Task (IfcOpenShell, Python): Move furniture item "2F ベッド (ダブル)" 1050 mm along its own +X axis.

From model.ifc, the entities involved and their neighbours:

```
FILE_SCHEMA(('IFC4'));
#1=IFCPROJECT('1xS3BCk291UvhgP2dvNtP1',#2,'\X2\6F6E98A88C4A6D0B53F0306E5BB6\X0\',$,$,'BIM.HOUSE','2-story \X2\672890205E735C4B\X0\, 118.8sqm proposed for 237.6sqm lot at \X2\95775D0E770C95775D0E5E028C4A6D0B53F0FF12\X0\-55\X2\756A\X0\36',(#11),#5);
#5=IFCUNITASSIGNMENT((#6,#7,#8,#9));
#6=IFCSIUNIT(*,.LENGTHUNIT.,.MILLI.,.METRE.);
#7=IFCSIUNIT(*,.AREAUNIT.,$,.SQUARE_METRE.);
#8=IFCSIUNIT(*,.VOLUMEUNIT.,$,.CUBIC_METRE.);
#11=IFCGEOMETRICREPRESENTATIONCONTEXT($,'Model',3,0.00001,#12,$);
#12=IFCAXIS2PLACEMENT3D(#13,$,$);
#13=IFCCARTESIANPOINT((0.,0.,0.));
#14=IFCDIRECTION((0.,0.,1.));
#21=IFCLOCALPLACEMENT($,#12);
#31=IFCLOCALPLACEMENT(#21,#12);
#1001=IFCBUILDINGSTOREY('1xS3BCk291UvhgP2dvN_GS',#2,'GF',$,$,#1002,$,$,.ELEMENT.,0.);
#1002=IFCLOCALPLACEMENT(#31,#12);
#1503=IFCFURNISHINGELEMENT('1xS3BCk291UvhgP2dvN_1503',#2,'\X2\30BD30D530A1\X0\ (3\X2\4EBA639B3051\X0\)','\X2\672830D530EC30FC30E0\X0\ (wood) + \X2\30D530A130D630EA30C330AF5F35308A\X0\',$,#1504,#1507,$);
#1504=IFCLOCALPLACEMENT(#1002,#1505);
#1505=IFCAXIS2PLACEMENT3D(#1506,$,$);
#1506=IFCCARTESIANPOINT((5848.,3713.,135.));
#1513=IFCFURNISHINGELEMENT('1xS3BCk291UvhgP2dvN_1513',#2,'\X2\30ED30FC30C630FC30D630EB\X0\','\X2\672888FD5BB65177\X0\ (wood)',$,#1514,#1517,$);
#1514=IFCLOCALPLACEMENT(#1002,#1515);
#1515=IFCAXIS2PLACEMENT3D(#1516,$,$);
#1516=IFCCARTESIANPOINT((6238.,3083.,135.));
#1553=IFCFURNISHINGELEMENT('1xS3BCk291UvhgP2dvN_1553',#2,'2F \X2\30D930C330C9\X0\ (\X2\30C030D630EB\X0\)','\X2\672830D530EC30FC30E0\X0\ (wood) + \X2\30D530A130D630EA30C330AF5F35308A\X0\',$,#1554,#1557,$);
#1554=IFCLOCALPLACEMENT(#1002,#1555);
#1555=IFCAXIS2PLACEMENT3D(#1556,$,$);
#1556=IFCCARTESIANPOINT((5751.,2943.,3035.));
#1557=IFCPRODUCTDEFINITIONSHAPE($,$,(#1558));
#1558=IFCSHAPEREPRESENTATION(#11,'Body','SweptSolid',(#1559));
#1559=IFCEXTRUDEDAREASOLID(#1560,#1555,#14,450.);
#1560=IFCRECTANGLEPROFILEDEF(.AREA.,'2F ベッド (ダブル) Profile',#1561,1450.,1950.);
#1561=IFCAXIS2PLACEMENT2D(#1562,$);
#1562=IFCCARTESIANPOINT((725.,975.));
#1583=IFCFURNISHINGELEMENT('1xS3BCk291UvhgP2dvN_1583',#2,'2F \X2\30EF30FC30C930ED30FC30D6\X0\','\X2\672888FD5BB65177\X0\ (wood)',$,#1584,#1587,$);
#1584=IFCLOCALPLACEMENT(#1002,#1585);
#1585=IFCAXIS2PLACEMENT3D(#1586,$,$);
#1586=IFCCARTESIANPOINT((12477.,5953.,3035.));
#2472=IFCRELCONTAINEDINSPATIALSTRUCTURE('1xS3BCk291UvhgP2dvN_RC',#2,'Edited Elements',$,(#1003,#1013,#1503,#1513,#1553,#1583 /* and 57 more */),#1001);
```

```python
import ifcopenshell
import ifcopenshell.api.geometry
import ifcopenshell.util.placement
import ifcopenshell.util.unit

model = ifcopenshell.open("model.ifc")
unit_scale = ifcopenshell.util.unit.calculate_unit_scale(model)

item = model.by_guid("1xS3BCk291UvhgP2dvN_1553")
matrix = ifcopenshell.util.placement.get_local_placement(item.ObjectPlacement)
matrix[:3, 3] += matrix[:3, 0] * 1.05 / unit_scale
ifcopenshell.api.geometry.edit_object_placement(model, product=item, matrix=matrix, is_si=False)

print(ifcopenshell.util.placement.get_local_placement(item.ObjectPlacement).round(3) + 0.0)

model.write("model_rev.ifc")
```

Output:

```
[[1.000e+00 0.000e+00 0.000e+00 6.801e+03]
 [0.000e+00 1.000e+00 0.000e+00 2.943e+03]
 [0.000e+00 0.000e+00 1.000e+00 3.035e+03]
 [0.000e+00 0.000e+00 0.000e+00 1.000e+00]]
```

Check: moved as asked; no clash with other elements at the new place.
